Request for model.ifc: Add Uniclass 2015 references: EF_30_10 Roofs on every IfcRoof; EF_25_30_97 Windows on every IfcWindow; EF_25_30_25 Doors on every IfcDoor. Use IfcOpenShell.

First a look at what the model holds.

```python
import ifcopenshell

model = ifcopenshell.open("model.ifc")
print(model.schema)
print("classifications:", [c.Name for c in model.by_type("IfcClassification")])
for ifc_class in ("IfcDoor", "IfcRoof", "IfcStair", "IfcWall", "IfcWindow"):
    print(ifc_class, len(model.by_type(ifc_class)))
```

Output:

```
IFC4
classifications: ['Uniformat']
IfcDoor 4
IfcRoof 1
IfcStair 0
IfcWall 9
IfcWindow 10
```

```python
import ifcopenshell
import ifcopenshell.api.classification

model = ifcopenshell.open("model.ifc")

system = ifcopenshell.api.classification.add_classification(model, classification="Uniclass 2015")

codes = {
    "IfcRoof": ("EF_30_10", "Roofs"),
    "IfcWindow": ("EF_25_30_97", "Windows"),
    "IfcDoor": ("EF_25_30_25", "Doors"),
}
for ifc_class, (code, name) in codes.items():
    products = model.by_type(ifc_class)
    ifcopenshell.api.classification.add_reference(
        model, products=products, classification=system, identification=code, name=name
    )
    print(code, len(products))

model.write("model_v2.ifc")
```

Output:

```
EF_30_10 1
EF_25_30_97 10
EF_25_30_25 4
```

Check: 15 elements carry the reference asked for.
